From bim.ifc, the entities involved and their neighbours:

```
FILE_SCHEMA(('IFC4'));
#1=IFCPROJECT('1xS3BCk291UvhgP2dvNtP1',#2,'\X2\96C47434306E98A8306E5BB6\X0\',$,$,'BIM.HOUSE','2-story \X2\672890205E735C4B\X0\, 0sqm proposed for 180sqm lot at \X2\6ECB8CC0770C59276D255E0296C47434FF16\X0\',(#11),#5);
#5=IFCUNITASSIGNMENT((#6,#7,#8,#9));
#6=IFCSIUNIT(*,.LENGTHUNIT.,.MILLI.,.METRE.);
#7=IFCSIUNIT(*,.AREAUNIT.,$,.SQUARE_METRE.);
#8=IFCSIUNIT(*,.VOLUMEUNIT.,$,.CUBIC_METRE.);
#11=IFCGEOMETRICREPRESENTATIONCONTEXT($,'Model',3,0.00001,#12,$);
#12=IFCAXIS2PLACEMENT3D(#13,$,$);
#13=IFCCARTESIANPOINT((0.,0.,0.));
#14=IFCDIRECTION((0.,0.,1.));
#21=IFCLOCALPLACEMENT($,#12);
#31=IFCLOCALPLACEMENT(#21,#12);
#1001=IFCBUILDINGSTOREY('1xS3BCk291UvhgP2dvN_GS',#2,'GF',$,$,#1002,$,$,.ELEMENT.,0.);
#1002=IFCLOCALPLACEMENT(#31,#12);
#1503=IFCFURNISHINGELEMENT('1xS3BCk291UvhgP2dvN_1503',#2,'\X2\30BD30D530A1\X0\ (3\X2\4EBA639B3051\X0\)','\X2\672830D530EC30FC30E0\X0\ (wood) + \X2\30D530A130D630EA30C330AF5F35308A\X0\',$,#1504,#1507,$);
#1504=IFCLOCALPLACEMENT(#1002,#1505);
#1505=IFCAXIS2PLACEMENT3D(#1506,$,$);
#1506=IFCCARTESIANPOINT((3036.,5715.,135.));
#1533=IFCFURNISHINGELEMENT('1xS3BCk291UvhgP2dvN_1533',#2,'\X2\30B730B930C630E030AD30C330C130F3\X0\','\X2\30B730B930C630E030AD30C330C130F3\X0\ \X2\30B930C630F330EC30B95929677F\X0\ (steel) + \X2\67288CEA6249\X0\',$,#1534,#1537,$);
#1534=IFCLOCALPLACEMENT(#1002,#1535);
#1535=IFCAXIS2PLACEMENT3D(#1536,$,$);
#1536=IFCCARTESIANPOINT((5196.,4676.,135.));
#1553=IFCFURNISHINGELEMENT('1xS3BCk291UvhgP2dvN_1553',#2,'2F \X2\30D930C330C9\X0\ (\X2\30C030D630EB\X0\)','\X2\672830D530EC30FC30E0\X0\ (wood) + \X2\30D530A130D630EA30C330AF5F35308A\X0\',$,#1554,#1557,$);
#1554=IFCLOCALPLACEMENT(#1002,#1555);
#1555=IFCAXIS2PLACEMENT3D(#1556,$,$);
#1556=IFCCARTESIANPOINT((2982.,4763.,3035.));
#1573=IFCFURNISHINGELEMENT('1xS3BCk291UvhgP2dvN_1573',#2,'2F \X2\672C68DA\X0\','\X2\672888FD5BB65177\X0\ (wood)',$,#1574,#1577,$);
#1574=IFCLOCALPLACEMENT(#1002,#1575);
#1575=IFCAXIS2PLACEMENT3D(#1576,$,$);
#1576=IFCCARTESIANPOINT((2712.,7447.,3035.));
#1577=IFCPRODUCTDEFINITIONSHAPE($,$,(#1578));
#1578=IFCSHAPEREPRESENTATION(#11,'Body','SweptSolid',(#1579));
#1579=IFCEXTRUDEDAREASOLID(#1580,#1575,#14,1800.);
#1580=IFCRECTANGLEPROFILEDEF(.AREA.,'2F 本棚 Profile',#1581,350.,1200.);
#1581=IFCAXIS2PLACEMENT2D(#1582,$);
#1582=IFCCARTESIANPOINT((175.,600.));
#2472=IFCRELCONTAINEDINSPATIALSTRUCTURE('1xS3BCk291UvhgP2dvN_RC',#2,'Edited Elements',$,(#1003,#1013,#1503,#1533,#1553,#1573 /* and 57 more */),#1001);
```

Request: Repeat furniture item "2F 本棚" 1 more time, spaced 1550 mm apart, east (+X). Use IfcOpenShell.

```python
import numpy as np
import ifcopenshell
import ifcopenshell.api.geometry
import ifcopenshell.api.root
import ifcopenshell.util.element
import ifcopenshell.util.placement
import ifcopenshell.util.unit

model = ifcopenshell.open("bim.ifc")
unit_scale = ifcopenshell.util.unit.calculate_unit_scale(model)


def reuse_history(source, copy):
    """copy_class also copies each property set's owner history, people and application; keep the originals."""
    for rel in copy.IsDefinedBy:
        if rel.is_a("IfcRelDefinesByProperties") and (history := rel.RelatingPropertyDefinition.OwnerHistory):
            rel.RelatingPropertyDefinition.OwnerHistory = source.OwnerHistory
            ifcopenshell.util.element.remove_deep2(model, history)


source = model.by_guid("1xS3BCk291UvhgP2dvN_1573")
base = ifcopenshell.util.placement.get_local_placement(source.ObjectPlacement)
step = np.array([1.0, 0.0, 0.0]) * 1.55 / unit_scale

for i in range(1, 2):
    copy = ifcopenshell.api.root.copy_class(model, product=source)
    copy.Representation = ifcopenshell.util.element.copy_deep(
        model, source.Representation, exclude=["IfcGeometricRepresentationContext", "IfcRepresentationMap"]
    )
    reuse_history(source, copy)
    matrix = base.copy()
    matrix[:3, 3] += i * step
    print("added at", matrix[:3, 3].round(3) + 0.0)
    ifcopenshell.api.geometry.edit_object_placement(model, product=copy, matrix=matrix, is_si=False)

model.write("bim_rev.ifc")
```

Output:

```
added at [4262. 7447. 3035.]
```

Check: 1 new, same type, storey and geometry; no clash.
